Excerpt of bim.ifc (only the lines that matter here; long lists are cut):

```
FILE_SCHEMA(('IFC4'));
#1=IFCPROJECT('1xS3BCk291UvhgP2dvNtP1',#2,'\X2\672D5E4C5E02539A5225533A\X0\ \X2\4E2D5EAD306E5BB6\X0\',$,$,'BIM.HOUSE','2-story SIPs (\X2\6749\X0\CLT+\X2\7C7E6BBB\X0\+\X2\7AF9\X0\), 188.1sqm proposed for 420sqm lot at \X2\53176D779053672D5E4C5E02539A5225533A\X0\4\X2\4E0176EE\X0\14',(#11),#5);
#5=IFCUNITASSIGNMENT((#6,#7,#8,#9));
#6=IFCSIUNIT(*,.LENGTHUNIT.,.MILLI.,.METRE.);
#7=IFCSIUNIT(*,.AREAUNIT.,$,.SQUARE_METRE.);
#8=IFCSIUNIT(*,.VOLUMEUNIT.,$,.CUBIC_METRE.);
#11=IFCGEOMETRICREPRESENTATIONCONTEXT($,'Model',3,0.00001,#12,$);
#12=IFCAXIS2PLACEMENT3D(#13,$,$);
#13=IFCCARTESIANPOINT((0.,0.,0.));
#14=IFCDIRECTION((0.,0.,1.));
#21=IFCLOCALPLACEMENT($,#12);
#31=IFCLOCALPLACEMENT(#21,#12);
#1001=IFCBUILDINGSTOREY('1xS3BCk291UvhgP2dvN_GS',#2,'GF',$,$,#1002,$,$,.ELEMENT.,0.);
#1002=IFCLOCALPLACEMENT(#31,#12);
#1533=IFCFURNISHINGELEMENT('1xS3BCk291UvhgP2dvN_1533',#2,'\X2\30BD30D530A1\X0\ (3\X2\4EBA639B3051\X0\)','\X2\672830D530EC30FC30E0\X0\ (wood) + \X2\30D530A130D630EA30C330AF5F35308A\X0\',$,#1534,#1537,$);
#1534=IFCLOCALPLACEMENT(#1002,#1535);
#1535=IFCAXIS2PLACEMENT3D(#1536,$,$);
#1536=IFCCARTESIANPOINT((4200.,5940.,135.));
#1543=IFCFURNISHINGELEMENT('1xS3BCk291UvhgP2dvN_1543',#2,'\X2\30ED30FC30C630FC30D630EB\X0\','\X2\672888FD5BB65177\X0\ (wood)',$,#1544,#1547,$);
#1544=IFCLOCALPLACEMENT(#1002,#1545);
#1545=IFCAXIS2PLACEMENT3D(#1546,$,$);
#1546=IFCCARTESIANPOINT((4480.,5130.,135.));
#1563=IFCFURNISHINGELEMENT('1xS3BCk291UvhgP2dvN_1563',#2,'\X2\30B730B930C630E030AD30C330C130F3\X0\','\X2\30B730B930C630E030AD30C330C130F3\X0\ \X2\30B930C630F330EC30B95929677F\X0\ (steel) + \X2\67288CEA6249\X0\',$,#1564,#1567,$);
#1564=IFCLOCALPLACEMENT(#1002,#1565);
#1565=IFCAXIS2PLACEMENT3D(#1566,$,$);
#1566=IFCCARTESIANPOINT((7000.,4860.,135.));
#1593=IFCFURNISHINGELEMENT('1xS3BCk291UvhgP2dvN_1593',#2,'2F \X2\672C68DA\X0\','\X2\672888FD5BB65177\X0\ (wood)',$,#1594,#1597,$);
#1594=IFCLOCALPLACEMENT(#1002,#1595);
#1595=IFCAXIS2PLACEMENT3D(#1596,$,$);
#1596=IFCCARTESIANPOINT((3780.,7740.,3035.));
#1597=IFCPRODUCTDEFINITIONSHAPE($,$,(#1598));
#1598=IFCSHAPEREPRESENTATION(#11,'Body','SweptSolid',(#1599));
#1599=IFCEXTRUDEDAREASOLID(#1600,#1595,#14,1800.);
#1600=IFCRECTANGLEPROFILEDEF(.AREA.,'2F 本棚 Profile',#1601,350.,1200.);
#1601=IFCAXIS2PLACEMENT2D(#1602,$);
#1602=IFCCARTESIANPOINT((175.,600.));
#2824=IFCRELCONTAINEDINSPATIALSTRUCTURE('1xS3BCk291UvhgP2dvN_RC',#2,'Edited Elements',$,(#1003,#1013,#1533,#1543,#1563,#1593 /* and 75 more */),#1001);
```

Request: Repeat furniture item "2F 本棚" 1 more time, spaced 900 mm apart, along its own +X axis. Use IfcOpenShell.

```python
import ifcopenshell
import ifcopenshell.api.geometry
import ifcopenshell.api.root
import ifcopenshell.util.element
import ifcopenshell.util.placement

model = ifcopenshell.open("bim.ifc")


def reuse_history(source, copy):
    """copy_class also copies each property set's owner history, people and application; keep the originals."""
    for rel in copy.IsDefinedBy:
        if rel.is_a("IfcRelDefinesByProperties") and (history := rel.RelatingPropertyDefinition.OwnerHistory):
            rel.RelatingPropertyDefinition.OwnerHistory = source.OwnerHistory
            ifcopenshell.util.element.remove_deep2(model, history)


source = model.by_id(1593)
base = ifcopenshell.util.placement.get_local_placement(source.ObjectPlacement)
step = base[:3, 0] * 900.0

for i in range(1, 2):
    copy = ifcopenshell.api.root.copy_class(model, product=source)
    copy.Representation = ifcopenshell.util.element.copy_deep(
        model, source.Representation, exclude=["IfcGeometricRepresentationContext", "IfcRepresentationMap"]
    )
    reuse_history(source, copy)
    matrix = base.copy()
    matrix[:3, 3] += i * step
    print("added at", matrix[:3, 3].round(3) + 0.0)
    ifcopenshell.api.geometry.edit_object_placement(model, product=copy, matrix=matrix, is_si=False)

model.write("bim-out.ifc")
```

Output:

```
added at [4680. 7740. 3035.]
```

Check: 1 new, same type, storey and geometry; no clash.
